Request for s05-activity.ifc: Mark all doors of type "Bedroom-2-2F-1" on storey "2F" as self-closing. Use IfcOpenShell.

First a look at what the model holds.

```python
import ifcopenshell
import ifcopenshell.util.element

model = ifcopenshell.open("s05-activity.ifc")
print(model.schema)
storey = next(s for s in model.by_type("IfcBuildingStorey") if s.Name == "2F")
doors = [e for e in ifcopenshell.util.element.get_decomposition(storey) if e.is_a("IfcDoor")]
seen = {}
for e in doors:
    element_type = ifcopenshell.util.element.get_type(e)
    key = (element_type.Name if element_type != e and element_type else None, ifcopenshell.util.element.get_pset(e, "Pset_DoorCommon", "SelfClosing"))
    seen[key] = seen.get(key, 0) + 1
for (name, value), count in sorted(seen.items(), key=str):
    print(count, "x", name, "|", value)
```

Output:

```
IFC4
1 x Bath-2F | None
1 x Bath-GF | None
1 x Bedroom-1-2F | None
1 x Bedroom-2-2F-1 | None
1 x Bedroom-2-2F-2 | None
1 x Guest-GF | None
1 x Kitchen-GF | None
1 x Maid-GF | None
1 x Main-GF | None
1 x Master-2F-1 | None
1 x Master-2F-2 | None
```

```python
import ifcopenshell
import ifcopenshell.api.pset
import ifcopenshell.util.element

model = ifcopenshell.open("s05-activity.ifc")

storey = next(s for s in model.by_type("IfcBuildingStorey") if s.Name == "2F")
doors = [e for e in ifcopenshell.util.element.get_decomposition(storey) if e.is_a("IfcDoor")]

count = 0
for e in doors:
    element_type = ifcopenshell.util.element.get_type(e)
    if element_type in (None, e) or element_type.Name != "Bedroom-2-2F-1":
        continue
    # add_pset returns the element's existing set when there is one.
    pset = ifcopenshell.api.pset.add_pset(model, product=e, name="Pset_DoorCommon")
    ifcopenshell.api.pset.edit_pset(model, pset=pset, properties={"SelfClosing": True})
    count += 1

print(count, "doors updated")

model.write("s05-activity_updated.ifc")
```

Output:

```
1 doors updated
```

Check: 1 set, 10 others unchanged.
